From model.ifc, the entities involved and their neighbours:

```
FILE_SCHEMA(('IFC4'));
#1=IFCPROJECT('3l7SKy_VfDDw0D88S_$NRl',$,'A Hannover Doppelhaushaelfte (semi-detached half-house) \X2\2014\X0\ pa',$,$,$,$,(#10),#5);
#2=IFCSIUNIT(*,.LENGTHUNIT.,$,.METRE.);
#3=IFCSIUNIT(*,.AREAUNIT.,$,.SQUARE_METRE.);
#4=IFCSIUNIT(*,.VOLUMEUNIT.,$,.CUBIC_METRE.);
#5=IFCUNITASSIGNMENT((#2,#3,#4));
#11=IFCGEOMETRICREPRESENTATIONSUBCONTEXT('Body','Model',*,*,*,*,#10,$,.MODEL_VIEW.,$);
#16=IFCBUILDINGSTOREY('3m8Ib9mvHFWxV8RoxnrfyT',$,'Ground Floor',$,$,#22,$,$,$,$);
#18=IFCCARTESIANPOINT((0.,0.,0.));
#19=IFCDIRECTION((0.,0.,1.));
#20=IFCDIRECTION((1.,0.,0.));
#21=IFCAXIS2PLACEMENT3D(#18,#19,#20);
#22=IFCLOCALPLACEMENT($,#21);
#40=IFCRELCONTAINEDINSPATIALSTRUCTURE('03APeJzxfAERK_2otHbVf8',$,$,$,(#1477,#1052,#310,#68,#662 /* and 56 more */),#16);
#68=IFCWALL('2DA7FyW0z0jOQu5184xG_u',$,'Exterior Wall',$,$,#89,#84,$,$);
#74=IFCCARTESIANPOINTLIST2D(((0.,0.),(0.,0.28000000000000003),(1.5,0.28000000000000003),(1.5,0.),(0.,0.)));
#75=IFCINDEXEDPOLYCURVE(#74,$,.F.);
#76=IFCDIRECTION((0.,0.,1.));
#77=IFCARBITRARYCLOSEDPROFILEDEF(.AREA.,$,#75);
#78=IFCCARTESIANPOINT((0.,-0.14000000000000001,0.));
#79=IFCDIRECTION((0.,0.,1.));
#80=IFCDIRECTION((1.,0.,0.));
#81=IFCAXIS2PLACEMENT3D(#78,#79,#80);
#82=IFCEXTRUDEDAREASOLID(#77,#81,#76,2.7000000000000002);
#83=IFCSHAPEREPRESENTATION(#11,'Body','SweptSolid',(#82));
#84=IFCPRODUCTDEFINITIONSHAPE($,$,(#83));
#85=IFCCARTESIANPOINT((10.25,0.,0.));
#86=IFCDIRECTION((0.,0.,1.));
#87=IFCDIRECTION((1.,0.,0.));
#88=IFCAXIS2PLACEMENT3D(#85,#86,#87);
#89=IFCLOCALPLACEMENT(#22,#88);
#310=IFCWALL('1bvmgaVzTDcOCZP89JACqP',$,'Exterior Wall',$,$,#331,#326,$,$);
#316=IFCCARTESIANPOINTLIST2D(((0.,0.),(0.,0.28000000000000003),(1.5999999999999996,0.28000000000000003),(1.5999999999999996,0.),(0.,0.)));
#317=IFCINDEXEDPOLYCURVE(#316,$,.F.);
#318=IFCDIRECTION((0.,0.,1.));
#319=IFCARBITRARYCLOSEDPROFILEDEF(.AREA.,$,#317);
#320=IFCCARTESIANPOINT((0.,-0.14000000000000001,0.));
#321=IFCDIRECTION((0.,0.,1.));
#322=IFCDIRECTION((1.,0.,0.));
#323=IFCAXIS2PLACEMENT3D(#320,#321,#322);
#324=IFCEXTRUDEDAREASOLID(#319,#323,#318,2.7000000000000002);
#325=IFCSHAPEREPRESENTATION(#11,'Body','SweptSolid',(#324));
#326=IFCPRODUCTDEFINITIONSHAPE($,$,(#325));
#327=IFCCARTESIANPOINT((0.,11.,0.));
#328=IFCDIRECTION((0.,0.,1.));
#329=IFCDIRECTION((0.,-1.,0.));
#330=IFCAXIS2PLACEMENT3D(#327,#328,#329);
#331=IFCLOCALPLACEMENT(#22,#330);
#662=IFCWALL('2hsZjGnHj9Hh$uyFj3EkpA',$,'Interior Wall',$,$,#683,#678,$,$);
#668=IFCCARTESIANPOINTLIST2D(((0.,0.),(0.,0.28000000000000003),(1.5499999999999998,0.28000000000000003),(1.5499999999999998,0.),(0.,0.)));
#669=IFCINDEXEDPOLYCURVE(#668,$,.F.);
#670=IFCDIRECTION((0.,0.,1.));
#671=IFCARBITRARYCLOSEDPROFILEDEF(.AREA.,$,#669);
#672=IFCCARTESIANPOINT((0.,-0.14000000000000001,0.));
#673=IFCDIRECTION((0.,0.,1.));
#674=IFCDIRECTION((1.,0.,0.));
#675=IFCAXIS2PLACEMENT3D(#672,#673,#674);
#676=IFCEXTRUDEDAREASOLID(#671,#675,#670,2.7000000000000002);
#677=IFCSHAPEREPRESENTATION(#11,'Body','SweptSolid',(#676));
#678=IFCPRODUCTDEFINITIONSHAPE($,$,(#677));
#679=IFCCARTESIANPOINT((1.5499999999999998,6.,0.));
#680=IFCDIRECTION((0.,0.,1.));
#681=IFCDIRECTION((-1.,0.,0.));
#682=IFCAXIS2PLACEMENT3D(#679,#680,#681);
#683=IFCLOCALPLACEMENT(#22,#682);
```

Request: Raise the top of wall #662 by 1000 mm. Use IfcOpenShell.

```python
import ifcopenshell
import ifcopenshell.geom
import ifcopenshell.util.representation
import ifcopenshell.util.shape
import ifcopenshell.util.unit

model = ifcopenshell.open("model.ifc")
unit_scale = ifcopenshell.util.unit.calculate_unit_scale(model)
settings = ifcopenshell.geom.settings()


def volume(element):
    """Net volume in cubic metres, openings subtracted."""
    shape = ifcopenshell.geom.create_shape(settings, element)
    return ifcopenshell.util.shape.get_volume(shape.geometry)


wall = model.by_guid("2hsZjGnHj9Hh$uyFj3EkpA")
before = volume(wall)

body = ifcopenshell.util.representation.get_representation(wall, "Model", "Body")
solid = body.Items[0]
old_height = solid.Depth
solid.Depth += 1 / unit_scale
after = volume(wall)

print(f"height {old_height:g} -> {solid.Depth:g}, volume {before:.3f} -> {after:.3f} m3")

model.write("model_edited.ifc")
```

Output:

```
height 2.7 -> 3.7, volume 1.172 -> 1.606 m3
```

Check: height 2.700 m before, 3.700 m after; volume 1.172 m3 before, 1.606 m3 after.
